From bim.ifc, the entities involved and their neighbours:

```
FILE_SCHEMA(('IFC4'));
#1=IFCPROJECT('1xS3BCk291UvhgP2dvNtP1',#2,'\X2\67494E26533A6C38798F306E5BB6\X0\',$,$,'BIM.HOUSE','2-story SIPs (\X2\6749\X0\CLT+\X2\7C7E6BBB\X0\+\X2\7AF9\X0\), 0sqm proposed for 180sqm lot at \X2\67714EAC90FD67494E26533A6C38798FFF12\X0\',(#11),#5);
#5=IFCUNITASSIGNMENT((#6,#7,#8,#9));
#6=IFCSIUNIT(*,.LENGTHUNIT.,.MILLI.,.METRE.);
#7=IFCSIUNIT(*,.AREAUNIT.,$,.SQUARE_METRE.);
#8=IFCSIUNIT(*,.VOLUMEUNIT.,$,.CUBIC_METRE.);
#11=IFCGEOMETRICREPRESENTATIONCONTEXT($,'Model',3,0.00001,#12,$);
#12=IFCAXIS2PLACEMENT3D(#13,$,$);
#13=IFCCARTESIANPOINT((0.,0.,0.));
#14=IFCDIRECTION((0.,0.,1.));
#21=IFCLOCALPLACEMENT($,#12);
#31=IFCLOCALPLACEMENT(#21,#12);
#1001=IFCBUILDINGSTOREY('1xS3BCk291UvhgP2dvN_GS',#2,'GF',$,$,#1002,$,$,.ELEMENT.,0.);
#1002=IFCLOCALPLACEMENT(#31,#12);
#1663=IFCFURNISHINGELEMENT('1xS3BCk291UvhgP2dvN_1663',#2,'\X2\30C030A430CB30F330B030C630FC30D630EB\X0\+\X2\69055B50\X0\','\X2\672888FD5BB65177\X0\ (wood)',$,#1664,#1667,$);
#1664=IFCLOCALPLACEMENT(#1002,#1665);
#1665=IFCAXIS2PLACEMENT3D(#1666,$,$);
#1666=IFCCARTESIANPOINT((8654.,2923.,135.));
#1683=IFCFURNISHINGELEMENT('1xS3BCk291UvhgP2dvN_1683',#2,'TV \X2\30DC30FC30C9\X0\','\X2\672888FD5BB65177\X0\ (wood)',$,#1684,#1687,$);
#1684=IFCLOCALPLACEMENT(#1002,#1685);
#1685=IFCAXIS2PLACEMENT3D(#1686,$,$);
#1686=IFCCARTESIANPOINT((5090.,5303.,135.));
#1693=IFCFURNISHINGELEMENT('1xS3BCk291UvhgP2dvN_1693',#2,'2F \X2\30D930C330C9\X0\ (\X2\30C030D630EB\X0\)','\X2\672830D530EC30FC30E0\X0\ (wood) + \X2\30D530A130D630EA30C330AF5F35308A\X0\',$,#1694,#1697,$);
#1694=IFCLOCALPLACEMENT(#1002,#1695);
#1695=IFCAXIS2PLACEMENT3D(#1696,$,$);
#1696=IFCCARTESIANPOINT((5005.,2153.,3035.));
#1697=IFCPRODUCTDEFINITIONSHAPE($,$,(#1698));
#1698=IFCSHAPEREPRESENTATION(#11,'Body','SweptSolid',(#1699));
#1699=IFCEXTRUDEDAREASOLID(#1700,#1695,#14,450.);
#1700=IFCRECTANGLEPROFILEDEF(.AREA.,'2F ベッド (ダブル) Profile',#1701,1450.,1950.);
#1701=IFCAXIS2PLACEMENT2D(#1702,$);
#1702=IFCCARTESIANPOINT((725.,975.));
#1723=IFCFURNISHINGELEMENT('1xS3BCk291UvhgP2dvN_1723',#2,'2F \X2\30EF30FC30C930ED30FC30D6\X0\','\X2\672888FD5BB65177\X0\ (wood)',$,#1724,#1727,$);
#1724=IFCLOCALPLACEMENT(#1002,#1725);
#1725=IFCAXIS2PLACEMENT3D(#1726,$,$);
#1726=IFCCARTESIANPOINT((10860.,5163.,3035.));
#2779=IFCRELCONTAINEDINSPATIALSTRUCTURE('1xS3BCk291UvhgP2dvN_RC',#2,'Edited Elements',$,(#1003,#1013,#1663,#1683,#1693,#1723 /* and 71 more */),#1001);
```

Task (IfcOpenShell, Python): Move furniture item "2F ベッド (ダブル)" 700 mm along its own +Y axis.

```python
import ifcopenshell
import ifcopenshell.api.geometry
import ifcopenshell.util.placement

model = ifcopenshell.open("bim.ifc")

item = model.by_guid("1xS3BCk291UvhgP2dvN_1693")
matrix = ifcopenshell.util.placement.get_local_placement(item.ObjectPlacement)
matrix[:3, 3] += matrix[:3, 1] * 700.0
ifcopenshell.api.geometry.edit_object_placement(model, product=item, matrix=matrix, is_si=False)

print(ifcopenshell.util.placement.get_local_placement(item.ObjectPlacement).round(3) + 0.0)

model.write("bim_rev.ifc")
```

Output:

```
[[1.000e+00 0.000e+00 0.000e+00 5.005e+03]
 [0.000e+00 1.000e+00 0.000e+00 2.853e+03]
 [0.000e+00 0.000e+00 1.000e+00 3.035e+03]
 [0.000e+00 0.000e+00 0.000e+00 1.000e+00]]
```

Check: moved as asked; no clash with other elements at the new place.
